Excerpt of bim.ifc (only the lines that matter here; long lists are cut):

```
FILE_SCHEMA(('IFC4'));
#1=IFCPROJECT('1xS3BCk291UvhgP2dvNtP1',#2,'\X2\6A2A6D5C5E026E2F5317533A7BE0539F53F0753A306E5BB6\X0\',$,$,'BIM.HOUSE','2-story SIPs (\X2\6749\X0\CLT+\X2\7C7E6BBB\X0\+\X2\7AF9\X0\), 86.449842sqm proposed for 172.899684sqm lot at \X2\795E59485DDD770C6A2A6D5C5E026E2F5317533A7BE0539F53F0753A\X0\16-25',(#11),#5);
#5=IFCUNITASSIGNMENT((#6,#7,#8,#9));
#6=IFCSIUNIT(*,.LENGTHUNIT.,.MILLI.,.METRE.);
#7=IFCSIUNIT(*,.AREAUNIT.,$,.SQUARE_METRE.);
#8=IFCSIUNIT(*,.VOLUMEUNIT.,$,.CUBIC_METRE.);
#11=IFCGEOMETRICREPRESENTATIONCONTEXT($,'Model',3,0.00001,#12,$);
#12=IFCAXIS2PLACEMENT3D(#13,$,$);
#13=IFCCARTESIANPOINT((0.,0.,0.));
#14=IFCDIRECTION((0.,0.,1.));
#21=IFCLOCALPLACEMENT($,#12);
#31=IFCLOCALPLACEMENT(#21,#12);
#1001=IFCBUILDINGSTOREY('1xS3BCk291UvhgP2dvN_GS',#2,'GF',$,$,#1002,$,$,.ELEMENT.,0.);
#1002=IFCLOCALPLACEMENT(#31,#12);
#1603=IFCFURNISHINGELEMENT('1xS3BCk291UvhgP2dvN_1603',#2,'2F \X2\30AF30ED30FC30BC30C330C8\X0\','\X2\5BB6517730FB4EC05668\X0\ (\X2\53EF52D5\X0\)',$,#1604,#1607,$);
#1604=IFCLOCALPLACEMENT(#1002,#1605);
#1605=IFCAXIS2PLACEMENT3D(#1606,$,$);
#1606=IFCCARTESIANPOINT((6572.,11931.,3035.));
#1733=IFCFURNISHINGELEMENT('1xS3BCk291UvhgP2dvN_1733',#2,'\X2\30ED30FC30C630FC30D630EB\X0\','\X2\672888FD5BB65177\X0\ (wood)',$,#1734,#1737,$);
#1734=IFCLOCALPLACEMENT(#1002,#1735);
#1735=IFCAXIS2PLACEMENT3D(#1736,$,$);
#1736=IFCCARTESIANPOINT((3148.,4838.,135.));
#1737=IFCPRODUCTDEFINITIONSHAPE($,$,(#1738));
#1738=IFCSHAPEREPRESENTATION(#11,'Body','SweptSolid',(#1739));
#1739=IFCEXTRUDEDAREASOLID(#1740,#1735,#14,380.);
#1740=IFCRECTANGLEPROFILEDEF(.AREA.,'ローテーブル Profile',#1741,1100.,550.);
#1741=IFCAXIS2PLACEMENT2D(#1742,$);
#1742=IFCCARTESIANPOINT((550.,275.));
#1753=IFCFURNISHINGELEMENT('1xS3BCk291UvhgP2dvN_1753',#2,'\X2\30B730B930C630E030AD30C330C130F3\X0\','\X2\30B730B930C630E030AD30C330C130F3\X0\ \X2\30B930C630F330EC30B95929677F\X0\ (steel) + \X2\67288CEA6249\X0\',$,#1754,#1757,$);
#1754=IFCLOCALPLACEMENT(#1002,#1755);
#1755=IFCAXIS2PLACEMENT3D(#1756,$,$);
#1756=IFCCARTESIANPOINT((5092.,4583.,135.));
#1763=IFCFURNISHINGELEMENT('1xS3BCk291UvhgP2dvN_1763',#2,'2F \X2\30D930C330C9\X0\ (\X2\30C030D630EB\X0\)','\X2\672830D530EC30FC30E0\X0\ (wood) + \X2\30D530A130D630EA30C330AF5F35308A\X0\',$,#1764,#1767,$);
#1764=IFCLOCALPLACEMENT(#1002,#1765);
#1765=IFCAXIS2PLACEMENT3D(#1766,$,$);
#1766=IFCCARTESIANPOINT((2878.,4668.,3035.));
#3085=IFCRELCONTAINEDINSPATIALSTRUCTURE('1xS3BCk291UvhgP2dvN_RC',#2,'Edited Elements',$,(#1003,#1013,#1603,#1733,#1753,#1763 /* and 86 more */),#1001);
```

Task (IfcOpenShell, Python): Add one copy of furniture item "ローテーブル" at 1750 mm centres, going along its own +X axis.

```python
import ifcopenshell
import ifcopenshell.api.geometry
import ifcopenshell.api.root
import ifcopenshell.util.element
import ifcopenshell.util.placement
import ifcopenshell.util.unit

model = ifcopenshell.open("bim.ifc")
unit_scale = ifcopenshell.util.unit.calculate_unit_scale(model)


def reuse_history(source, copy):
    """copy_class also copies each property set's owner history, people and application; keep the originals."""
    for rel in copy.IsDefinedBy:
        if rel.is_a("IfcRelDefinesByProperties") and (history := rel.RelatingPropertyDefinition.OwnerHistory):
            rel.RelatingPropertyDefinition.OwnerHistory = source.OwnerHistory
            ifcopenshell.util.element.remove_deep2(model, history)


source = model.by_id(1733)
base = ifcopenshell.util.placement.get_local_placement(source.ObjectPlacement)
step = base[:3, 0] * 1.75 / unit_scale

for i in range(1, 2):
    copy = ifcopenshell.api.root.copy_class(model, product=source)
    copy.Representation = ifcopenshell.util.element.copy_deep(
        model, source.Representation, exclude=["IfcGeometricRepresentationContext", "IfcRepresentationMap"]
    )
    reuse_history(source, copy)
    matrix = base.copy()
    matrix[:3, 3] += i * step
    print("added at", matrix[:3, 3].round(3) + 0.0)
    ifcopenshell.api.geometry.edit_object_placement(model, product=copy, matrix=matrix, is_si=False)

model.write("bim_v2.ifc")
```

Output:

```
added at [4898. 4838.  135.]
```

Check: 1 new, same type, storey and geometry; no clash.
